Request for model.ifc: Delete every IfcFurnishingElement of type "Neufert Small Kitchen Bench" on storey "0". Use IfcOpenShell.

First a look at what the model holds.

```python
import ifcopenshell
import ifcopenshell.util.element

model = ifcopenshell.open("model.ifc")
print(model.schema)
storey = next(s for s in model.by_type("IfcBuildingStorey") if s.Name == "0")
furniture = [e for e in ifcopenshell.util.element.get_decomposition(storey) if e.is_a("IfcFurnishingElement")]
seen = {}
for e in furniture:
    element_type = ifcopenshell.util.element.get_type(e)
    name = element_type.Name if element_type not in (None, e) else None
    seen[name] = seen.get(name, 0) + 1
for name, count in sorted(seen.items(), key=str):
    print(count, "x", name)
```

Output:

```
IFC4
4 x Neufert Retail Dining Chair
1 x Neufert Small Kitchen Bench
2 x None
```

```python
import ifcopenshell
import ifcopenshell.api.root
import ifcopenshell.util.element

model = ifcopenshell.open("model.ifc")

storey = next(s for s in model.by_type("IfcBuildingStorey") if s.Name == "0")
furniture = [e for e in ifcopenshell.util.element.get_decomposition(storey) if e.is_a("IfcFurnishingElement")]
targets = [e for e in furniture if (t := ifcopenshell.util.element.get_type(e)) not in (None, e) and t.Name == "Neufert Small Kitchen Bench"]

for e in targets:
    ifcopenshell.api.root.remove_product(model, product=e)
print(len(targets), "removed")

model.write("model_v2.ifc")
```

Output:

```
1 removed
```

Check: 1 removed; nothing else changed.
